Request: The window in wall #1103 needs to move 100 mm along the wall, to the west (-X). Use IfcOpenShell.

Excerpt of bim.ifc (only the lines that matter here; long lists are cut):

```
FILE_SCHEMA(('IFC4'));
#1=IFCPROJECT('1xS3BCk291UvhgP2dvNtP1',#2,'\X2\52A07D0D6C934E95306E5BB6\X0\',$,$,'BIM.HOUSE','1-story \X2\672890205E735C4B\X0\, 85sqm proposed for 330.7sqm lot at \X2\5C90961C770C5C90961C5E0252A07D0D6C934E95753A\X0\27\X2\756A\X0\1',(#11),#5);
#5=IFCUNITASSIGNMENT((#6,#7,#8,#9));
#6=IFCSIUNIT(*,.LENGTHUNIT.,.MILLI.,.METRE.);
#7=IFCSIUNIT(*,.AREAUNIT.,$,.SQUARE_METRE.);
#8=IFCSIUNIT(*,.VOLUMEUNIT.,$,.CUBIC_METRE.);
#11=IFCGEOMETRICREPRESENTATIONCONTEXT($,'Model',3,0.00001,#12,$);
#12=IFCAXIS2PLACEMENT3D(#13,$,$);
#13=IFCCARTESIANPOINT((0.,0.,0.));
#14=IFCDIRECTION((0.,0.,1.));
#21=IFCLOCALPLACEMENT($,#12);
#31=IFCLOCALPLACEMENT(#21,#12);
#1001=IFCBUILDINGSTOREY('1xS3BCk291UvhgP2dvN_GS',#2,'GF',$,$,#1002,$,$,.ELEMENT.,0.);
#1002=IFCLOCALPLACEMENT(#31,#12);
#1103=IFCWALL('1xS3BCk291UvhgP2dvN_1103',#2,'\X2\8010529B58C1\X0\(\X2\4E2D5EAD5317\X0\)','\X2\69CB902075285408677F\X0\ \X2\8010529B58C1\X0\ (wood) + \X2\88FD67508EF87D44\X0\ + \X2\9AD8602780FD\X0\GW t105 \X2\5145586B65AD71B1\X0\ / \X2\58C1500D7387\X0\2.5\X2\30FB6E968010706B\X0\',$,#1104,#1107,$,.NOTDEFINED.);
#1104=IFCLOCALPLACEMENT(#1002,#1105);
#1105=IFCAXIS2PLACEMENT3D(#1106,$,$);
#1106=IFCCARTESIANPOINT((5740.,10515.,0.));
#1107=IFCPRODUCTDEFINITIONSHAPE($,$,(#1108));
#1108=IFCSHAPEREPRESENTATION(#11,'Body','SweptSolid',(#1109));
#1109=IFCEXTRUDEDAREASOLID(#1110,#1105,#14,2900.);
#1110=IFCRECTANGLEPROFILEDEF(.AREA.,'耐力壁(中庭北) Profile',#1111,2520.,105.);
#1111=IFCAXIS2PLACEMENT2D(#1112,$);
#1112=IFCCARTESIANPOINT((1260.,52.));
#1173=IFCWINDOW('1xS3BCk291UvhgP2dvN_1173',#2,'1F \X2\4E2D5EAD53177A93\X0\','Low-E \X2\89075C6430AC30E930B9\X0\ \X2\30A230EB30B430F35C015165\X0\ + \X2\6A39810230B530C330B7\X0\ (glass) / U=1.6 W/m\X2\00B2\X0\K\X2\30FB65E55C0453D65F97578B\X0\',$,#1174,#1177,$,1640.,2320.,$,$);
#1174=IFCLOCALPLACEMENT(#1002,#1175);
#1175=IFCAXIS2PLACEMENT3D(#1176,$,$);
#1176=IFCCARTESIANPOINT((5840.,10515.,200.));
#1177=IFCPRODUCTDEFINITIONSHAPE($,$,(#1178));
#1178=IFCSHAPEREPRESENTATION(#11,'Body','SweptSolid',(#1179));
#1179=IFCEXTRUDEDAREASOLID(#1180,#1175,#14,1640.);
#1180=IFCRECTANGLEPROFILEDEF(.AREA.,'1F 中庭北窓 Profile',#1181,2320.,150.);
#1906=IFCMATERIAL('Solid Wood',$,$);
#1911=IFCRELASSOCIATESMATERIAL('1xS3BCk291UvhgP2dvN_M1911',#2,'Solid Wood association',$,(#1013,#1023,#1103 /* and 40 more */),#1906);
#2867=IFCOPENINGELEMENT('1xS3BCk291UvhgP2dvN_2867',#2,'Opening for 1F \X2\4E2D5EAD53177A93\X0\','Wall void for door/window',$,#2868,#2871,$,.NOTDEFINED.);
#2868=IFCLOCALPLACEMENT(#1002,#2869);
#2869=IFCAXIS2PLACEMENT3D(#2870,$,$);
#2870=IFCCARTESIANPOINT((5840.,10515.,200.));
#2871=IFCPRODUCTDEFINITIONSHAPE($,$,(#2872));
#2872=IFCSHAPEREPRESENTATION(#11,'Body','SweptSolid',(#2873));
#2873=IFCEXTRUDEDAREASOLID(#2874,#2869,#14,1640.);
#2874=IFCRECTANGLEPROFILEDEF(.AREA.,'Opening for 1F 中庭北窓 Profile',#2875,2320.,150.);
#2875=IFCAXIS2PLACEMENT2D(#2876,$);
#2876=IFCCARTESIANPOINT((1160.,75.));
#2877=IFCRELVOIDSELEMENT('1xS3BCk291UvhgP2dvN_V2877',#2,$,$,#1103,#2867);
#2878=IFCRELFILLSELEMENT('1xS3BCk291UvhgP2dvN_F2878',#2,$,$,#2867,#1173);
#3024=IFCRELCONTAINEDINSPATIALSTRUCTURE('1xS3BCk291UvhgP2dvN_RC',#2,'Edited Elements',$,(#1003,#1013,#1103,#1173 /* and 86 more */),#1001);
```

```python
import ifcopenshell
import ifcopenshell.api.geometry
import ifcopenshell.util.placement
import ifcopenshell.util.unit

model = ifcopenshell.open("bim.ifc")
unit_scale = ifcopenshell.util.unit.calculate_unit_scale(model)

window = model.by_guid("1xS3BCk291UvhgP2dvN_1173")
opening = window.FillsVoids[0].RelatingOpeningElement
wall = opening.VoidsElements[0].RelatingBuildingElement

wall_matrix = ifcopenshell.util.placement.get_local_placement(wall.ObjectPlacement)
shift = wall_matrix[:3, 0] * -0.1 / unit_scale
before = ifcopenshell.util.placement.get_local_placement(window.ObjectPlacement)[:3, 3].copy()

# The window is not placed relative to its opening, so move both.
for product in (opening, window):
    matrix = ifcopenshell.util.placement.get_local_placement(product.ObjectPlacement)
    matrix[:3, 3] += shift
    ifcopenshell.api.geometry.edit_object_placement(model, product=product, matrix=matrix, is_si=False)

after = ifcopenshell.util.placement.get_local_placement(window.ObjectPlacement)[:3, 3]
print("window moved by", (after - before).round(3) + 0.0)

model.write("bim_rev.ifc")
```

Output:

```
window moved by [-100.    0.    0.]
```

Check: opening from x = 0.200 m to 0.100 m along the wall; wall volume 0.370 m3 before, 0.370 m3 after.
